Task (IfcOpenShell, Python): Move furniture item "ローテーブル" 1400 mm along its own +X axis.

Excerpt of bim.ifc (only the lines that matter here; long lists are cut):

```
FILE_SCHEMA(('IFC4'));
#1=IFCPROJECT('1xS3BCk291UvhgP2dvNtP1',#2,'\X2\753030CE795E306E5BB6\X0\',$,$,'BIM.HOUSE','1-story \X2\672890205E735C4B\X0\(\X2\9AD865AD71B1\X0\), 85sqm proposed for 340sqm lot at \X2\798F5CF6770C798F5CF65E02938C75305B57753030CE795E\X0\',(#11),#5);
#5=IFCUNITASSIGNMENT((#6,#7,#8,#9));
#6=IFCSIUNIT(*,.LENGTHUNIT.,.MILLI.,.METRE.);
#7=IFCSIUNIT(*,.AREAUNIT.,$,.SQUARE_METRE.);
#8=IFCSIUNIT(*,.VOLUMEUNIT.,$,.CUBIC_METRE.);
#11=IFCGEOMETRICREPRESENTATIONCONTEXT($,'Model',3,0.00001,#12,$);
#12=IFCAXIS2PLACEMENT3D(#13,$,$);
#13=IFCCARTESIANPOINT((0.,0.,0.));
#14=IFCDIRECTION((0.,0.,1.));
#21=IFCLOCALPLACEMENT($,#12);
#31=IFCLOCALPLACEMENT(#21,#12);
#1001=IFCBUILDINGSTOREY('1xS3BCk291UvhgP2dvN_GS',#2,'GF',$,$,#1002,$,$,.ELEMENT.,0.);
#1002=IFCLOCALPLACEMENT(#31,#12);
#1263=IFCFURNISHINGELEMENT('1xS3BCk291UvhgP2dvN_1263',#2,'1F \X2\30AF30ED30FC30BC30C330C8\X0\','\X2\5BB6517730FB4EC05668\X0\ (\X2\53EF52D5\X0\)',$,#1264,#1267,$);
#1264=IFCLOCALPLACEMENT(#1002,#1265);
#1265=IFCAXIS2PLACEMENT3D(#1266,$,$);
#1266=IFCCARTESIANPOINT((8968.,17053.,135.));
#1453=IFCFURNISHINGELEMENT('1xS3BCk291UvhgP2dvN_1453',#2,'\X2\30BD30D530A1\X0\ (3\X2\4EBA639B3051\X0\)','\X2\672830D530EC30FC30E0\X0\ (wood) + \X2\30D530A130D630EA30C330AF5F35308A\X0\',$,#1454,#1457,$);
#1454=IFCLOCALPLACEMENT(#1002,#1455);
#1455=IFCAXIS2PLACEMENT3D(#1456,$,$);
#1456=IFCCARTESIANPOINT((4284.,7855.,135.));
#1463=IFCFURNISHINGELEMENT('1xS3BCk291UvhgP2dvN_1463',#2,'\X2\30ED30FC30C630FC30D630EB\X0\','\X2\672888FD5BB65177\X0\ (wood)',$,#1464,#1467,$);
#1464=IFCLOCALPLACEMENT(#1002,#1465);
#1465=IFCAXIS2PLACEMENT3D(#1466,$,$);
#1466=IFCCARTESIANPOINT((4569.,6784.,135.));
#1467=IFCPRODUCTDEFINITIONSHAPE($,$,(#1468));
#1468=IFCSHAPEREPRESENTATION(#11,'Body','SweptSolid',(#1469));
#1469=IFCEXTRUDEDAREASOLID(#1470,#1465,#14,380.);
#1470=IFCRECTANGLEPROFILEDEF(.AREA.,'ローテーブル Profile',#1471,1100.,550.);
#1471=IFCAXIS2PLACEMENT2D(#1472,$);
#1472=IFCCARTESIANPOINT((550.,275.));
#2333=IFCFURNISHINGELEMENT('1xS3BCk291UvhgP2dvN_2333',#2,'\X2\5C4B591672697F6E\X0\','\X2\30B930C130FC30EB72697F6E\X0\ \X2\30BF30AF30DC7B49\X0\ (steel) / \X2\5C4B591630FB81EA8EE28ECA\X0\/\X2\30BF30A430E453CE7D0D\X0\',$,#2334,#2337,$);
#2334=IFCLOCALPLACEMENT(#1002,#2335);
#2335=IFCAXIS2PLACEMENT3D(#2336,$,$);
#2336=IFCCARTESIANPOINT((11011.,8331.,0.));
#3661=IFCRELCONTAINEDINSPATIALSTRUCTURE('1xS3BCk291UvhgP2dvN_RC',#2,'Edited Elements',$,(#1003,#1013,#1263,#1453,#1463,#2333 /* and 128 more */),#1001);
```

```python
import ifcopenshell
import ifcopenshell.api.geometry
import ifcopenshell.util.placement
import ifcopenshell.util.unit

model = ifcopenshell.open("bim.ifc")
unit_scale = ifcopenshell.util.unit.calculate_unit_scale(model)

item = model.by_id(1463)
matrix = ifcopenshell.util.placement.get_local_placement(item.ObjectPlacement)
matrix[:3, 3] += matrix[:3, 0] * 1.4 / unit_scale
ifcopenshell.api.geometry.edit_object_placement(model, product=item, matrix=matrix, is_si=False)

print(ifcopenshell.util.placement.get_local_placement(item.ObjectPlacement).round(3) + 0.0)

model.write("bim-out.ifc")
```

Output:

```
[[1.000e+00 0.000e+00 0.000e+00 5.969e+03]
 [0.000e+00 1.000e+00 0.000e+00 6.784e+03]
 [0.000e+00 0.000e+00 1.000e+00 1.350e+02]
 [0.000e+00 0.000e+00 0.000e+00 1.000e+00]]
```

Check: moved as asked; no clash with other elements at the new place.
